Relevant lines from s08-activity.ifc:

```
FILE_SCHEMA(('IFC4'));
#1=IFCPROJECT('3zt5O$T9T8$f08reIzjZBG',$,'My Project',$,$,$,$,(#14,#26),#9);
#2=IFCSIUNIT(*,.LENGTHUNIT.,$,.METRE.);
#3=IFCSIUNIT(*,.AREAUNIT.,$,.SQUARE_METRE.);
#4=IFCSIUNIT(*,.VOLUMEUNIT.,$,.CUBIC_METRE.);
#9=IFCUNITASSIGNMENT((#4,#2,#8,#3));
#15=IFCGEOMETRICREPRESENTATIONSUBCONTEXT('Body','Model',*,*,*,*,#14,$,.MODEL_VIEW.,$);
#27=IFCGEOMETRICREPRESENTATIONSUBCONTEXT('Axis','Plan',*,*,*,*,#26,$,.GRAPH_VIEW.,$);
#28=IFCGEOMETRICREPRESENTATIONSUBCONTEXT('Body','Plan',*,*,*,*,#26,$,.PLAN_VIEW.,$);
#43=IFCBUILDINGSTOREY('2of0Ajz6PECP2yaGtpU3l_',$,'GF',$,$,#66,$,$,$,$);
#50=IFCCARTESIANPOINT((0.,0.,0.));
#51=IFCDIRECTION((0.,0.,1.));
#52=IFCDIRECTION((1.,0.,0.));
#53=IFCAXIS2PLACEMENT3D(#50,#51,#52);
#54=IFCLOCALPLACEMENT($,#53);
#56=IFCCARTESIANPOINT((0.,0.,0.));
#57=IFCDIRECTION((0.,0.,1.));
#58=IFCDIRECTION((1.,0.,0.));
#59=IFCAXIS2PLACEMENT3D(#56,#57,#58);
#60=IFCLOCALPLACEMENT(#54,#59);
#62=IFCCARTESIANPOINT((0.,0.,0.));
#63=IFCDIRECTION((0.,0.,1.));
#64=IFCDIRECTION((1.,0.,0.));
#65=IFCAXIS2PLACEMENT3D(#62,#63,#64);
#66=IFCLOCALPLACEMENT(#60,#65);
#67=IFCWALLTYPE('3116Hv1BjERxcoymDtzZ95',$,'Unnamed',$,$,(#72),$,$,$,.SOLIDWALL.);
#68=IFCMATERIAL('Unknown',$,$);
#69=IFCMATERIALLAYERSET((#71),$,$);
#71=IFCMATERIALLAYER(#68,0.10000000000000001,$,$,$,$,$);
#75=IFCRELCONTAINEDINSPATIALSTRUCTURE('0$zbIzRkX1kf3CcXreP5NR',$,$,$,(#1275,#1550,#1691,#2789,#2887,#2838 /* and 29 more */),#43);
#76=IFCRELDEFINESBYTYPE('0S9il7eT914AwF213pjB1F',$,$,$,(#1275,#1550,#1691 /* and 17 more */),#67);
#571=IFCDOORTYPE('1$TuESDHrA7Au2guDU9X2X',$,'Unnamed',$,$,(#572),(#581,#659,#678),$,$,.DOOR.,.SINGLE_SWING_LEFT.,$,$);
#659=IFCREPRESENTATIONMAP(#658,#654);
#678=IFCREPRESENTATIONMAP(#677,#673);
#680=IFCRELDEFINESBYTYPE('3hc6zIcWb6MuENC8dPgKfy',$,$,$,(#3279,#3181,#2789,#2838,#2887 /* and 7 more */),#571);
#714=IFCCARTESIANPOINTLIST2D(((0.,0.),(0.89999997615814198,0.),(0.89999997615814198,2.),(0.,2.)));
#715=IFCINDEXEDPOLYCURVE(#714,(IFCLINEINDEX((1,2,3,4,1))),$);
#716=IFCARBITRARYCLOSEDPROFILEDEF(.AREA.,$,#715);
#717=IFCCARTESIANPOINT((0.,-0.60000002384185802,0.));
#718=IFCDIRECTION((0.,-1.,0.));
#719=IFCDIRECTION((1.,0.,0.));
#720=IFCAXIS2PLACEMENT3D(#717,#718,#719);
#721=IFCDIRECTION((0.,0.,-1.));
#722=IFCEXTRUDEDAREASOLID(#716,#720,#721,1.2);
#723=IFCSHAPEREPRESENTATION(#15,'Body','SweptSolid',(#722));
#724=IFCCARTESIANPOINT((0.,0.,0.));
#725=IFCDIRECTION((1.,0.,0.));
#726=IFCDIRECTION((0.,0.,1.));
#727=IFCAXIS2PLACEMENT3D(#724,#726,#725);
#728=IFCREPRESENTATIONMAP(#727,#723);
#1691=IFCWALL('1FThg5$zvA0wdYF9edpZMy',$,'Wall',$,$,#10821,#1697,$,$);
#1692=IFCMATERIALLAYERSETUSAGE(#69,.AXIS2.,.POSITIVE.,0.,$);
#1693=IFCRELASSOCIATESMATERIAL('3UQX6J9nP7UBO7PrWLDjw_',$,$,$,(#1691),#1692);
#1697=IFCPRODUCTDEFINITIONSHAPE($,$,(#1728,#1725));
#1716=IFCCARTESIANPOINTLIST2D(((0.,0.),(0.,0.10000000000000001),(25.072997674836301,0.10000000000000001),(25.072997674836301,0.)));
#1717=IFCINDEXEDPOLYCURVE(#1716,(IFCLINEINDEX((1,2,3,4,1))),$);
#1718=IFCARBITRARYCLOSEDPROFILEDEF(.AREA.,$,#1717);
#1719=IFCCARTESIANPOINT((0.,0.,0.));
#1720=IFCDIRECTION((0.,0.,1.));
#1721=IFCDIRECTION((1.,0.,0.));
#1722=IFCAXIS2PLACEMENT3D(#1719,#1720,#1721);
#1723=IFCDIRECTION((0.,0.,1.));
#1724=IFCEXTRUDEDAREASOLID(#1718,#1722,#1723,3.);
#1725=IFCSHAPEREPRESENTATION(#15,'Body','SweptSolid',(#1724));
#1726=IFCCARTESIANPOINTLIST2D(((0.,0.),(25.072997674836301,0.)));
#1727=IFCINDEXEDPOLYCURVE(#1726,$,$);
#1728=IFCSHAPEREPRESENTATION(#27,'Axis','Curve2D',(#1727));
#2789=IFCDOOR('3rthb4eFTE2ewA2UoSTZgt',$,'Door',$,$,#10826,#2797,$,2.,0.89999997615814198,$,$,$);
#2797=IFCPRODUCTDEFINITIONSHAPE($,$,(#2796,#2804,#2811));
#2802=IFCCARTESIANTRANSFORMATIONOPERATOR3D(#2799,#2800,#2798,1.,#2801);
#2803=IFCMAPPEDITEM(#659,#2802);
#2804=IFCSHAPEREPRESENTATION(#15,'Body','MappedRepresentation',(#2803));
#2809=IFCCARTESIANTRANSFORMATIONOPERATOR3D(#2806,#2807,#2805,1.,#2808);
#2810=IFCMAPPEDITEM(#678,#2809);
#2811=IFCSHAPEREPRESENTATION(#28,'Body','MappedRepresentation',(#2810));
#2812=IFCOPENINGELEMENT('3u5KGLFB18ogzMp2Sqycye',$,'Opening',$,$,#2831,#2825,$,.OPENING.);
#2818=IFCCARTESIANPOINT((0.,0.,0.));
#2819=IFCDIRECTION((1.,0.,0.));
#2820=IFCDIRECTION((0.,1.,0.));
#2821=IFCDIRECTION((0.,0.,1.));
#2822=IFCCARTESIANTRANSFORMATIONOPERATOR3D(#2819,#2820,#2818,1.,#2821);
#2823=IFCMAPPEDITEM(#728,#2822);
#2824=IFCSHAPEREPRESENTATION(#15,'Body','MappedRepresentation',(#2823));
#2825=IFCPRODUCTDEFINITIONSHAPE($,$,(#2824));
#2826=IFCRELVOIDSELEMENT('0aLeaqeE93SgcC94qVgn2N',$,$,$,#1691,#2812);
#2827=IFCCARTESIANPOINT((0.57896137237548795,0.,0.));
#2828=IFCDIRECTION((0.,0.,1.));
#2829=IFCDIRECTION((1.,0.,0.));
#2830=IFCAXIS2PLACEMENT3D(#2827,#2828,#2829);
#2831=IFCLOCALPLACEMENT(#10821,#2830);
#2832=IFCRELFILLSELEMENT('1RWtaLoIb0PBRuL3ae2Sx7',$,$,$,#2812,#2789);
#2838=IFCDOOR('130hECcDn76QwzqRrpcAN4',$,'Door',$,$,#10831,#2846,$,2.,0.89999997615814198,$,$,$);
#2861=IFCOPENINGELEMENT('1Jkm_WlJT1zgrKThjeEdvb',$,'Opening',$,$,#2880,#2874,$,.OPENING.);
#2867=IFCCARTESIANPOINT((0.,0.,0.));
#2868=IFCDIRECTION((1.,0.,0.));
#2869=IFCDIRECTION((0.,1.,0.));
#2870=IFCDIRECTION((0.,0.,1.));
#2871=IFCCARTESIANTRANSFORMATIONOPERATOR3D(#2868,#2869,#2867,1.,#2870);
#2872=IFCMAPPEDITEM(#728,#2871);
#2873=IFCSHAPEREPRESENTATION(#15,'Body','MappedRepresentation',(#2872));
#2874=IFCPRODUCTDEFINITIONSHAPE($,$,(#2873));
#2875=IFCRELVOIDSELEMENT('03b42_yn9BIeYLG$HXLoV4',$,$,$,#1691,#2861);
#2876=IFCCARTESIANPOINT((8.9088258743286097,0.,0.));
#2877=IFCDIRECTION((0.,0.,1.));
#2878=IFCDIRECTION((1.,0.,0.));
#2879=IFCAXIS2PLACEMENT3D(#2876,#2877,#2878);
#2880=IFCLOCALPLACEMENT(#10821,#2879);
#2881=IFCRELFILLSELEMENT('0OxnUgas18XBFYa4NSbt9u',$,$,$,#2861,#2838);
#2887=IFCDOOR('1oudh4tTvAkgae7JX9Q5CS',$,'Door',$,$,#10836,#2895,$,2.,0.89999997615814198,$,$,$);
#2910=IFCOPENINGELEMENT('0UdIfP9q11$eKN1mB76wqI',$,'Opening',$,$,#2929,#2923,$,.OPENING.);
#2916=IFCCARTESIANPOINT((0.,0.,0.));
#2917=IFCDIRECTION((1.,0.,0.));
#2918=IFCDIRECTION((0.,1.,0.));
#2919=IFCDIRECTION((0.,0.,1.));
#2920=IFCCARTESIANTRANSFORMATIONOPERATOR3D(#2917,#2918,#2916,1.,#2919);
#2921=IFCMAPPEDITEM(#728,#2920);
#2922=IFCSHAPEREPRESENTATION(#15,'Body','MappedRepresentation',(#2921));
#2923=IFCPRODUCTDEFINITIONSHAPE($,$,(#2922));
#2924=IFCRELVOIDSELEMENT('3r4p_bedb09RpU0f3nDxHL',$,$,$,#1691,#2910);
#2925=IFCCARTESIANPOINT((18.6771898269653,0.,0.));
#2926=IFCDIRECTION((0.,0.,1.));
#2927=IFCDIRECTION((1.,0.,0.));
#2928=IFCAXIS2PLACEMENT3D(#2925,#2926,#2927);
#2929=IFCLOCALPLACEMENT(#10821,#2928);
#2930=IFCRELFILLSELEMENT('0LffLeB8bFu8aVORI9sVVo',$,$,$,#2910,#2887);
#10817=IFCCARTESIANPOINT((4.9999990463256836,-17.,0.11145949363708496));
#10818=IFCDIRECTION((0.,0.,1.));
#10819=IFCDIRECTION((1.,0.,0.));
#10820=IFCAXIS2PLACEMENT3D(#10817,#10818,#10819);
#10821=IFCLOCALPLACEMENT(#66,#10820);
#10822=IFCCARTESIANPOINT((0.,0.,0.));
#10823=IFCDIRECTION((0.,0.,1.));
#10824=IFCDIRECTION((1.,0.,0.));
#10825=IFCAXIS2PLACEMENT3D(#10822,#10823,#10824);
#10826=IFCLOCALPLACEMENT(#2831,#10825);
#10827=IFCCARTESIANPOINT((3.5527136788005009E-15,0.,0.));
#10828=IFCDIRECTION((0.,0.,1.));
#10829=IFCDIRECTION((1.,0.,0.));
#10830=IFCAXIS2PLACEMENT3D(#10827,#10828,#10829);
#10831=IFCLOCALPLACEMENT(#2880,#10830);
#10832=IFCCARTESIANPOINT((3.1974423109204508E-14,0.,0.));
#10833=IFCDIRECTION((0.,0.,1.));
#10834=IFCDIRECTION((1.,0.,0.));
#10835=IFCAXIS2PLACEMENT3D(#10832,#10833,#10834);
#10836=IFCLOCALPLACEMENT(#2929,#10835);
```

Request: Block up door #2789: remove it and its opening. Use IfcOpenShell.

```python
import ifcopenshell
import ifcopenshell.api.feature
import ifcopenshell.api.root
import ifcopenshell.geom
import ifcopenshell.util.shape

model = ifcopenshell.open("s08-activity.ifc")
settings = ifcopenshell.geom.settings()


def volume(element):
    """Net volume in cubic metres, openings subtracted."""
    shape = ifcopenshell.geom.create_shape(settings, element)
    return ifcopenshell.util.shape.get_volume(shape.geometry)


door = model.by_guid("3rthb4eFTE2ewA2UoSTZgt")
opening = door.FillsVoids[0].RelatingOpeningElement
wall = opening.VoidsElements[0].RelatingBuildingElement
before = volume(wall)

ifcopenshell.api.root.remove_product(model, product=door)
ifcopenshell.api.feature.remove_feature(model, feature=opening)

after = volume(wall)

print(f"wall volume {before:.3f} -> {after:.3f} m3")

model.write("s08-activity_edited.ifc")
```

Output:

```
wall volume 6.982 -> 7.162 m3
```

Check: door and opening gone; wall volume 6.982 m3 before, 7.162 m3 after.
